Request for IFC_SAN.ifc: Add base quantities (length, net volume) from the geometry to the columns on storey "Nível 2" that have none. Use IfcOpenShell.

First a look at what the model holds.

```python
import ifcopenshell
import ifcopenshell.util.element
import ifcopenshell.util.unit

model = ifcopenshell.open("IFC_SAN.ifc")
print(model.schema)
for unit_type in ("LENGTHUNIT", "AREAUNIT", "VOLUMEUNIT"):
    print(unit_type, ifcopenshell.util.unit.calculate_unit_scale(model, unit_type))
storey = next(s for s in model.by_type("IfcBuildingStorey") if s.Name == "Nível 2")
columns = [e for e in ifcopenshell.util.element.get_decomposition(storey) if e.is_a("IfcColumn")]
for e in sorted(columns, key=lambda e: e.id()):
    print(e.id(), e.is_a(), e.Name, list(ifcopenshell.util.element.get_psets(e, qtos_only=True)), sep=" | ")
```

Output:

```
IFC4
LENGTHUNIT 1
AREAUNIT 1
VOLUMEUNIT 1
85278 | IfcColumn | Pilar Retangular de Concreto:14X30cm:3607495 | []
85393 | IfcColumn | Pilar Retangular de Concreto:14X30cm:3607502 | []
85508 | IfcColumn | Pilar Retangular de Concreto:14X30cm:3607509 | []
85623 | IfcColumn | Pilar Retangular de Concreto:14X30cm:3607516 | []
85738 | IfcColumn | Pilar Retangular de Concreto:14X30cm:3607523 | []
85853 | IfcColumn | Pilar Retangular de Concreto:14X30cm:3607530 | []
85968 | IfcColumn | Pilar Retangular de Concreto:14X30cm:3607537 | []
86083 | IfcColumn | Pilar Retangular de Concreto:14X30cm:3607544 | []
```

```python
import ifcopenshell
import ifcopenshell.api.pset
import ifcopenshell.geom
import ifcopenshell.util.element
import ifcopenshell.util.shape
import ifcopenshell.util.unit

model = ifcopenshell.open("IFC_SAN.ifc")
unit_scale = ifcopenshell.util.unit.calculate_unit_scale(model)
volume_scale = ifcopenshell.util.unit.calculate_unit_scale(model, "VOLUMEUNIT")
settings = ifcopenshell.geom.settings()

storey = next(s for s in model.by_type("IfcBuildingStorey") if s.Name == "Nível 2")
columns = [e for e in ifcopenshell.util.element.get_decomposition(storey) if e.is_a("IfcColumn")]

for e in sorted(columns, key=lambda e: e.id()):
    if ifcopenshell.util.element.get_psets(e, qtos_only=True, should_inherit=False):
        continue
    # Geometry comes back in metres, in the element's own axes.
    shape = ifcopenshell.geom.create_shape(settings, e)
    values = {
        "Length": ifcopenshell.util.shape.get_z(shape.geometry) / unit_scale,
        "NetVolume": ifcopenshell.util.shape.get_volume(shape.geometry) / volume_scale,
    }
    qto = ifcopenshell.api.pset.add_qto(model, product=e, name="Qto_ColumnBaseQuantities")
    ifcopenshell.api.pset.edit_qto(model, qto=qto, properties=values)
    print(e.id(), {k: round(v, 3) for k, v in values.items()})

model.write("IFC_SAN_updated.ifc")
```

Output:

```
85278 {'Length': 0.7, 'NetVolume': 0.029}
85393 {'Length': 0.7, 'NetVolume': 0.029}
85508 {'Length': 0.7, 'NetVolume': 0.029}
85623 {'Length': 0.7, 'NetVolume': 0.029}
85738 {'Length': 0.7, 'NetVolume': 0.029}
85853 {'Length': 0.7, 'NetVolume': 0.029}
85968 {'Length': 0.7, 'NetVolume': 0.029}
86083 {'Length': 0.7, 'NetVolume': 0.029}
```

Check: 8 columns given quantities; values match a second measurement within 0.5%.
